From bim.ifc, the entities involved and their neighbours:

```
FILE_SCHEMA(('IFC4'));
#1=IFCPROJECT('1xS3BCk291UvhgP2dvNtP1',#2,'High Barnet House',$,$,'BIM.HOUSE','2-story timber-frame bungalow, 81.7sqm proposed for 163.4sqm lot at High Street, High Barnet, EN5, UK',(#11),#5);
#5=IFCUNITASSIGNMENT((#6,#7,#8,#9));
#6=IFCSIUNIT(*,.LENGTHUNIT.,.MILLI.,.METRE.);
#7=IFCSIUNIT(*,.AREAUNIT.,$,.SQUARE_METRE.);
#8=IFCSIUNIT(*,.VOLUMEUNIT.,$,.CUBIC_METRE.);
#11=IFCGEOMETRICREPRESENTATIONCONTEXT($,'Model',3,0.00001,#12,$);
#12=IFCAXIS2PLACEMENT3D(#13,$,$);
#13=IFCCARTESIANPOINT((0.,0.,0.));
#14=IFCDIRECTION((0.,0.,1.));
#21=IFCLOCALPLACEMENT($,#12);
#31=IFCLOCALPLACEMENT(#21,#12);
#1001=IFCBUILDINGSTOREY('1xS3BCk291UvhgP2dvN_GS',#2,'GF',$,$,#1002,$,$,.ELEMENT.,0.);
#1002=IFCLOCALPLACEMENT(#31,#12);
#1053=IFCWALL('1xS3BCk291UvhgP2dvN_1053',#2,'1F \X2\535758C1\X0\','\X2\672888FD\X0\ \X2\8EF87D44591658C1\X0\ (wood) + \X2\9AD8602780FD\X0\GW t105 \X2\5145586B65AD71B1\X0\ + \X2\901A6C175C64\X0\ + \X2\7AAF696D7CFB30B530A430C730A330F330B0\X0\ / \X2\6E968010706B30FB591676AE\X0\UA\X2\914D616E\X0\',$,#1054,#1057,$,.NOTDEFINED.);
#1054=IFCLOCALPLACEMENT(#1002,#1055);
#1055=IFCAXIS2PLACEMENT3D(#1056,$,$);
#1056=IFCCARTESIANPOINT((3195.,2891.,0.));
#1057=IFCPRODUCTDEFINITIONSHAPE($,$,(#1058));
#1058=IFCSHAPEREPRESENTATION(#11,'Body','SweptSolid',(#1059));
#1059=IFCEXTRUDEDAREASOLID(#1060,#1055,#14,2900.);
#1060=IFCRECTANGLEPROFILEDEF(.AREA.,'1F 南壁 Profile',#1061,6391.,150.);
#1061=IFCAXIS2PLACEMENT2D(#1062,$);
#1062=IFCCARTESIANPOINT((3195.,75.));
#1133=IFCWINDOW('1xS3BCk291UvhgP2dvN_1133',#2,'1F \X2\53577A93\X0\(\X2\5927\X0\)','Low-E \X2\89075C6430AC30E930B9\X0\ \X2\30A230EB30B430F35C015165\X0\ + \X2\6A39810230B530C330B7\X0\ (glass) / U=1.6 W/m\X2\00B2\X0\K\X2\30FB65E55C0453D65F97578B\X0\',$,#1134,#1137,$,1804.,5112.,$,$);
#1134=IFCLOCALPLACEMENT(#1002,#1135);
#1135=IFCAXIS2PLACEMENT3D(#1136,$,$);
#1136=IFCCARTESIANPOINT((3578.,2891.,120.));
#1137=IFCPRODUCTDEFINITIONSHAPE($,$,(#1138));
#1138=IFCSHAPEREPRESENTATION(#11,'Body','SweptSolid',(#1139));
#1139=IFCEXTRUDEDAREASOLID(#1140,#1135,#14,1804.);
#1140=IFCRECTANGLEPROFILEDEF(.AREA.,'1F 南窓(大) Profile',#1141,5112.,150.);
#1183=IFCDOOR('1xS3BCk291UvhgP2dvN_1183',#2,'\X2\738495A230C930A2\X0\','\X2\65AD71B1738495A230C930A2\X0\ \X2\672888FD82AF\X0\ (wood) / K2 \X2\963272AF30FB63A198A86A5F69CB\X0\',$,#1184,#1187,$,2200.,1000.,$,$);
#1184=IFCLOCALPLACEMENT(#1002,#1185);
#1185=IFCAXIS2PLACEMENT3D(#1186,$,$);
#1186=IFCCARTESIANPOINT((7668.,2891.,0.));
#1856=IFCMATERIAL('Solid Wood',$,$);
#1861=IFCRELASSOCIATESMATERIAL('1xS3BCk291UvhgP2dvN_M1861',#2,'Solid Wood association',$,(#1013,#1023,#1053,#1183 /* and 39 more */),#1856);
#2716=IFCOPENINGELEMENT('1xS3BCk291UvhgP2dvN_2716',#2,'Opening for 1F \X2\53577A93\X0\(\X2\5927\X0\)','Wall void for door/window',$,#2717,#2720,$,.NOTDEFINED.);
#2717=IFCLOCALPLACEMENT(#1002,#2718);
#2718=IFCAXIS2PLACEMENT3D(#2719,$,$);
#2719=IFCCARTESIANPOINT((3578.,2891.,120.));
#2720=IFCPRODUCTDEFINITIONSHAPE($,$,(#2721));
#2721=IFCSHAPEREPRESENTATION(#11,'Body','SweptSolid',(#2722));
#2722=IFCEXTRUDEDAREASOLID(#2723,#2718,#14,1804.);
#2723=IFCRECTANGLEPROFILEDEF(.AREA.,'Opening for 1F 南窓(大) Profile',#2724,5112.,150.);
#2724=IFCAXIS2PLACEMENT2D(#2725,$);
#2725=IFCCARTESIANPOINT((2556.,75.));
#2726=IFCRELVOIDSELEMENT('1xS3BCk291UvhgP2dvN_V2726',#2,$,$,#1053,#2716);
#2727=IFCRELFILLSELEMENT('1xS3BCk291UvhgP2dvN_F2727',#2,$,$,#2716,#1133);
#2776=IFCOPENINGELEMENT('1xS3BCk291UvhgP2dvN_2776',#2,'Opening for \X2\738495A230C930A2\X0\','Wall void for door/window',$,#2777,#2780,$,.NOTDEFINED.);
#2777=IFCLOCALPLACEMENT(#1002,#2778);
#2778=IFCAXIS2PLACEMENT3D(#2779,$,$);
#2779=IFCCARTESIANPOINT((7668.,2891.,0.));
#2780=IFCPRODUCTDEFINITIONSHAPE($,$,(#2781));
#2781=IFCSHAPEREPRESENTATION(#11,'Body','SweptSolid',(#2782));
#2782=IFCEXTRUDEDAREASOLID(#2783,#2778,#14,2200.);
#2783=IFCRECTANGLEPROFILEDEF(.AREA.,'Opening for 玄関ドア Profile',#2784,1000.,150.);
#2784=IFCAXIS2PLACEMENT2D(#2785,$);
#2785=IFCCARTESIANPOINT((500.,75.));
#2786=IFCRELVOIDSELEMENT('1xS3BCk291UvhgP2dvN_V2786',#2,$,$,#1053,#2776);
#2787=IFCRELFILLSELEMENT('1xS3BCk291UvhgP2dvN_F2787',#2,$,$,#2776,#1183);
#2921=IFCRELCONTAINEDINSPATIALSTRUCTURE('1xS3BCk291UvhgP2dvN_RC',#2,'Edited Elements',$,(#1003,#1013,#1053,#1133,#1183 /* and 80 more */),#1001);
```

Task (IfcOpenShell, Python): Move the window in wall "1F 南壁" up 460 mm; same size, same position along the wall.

```python
import numpy as np
import ifcopenshell
import ifcopenshell.api.geometry
import ifcopenshell.util.placement
import ifcopenshell.util.unit

model = ifcopenshell.open("bim.ifc")
unit_scale = ifcopenshell.util.unit.calculate_unit_scale(model)

window = model.by_guid("1xS3BCk291UvhgP2dvN_1133")
opening = window.FillsVoids[0].RelatingOpeningElement
dz = 0.46 / unit_scale

shift = np.array([0.0, 0.0, dz])
# The window is not placed relative to its opening, so move both.
for product in (opening, window):
    matrix = ifcopenshell.util.placement.get_local_placement(product.ObjectPlacement)
    matrix[:3, 3] += shift
    ifcopenshell.api.geometry.edit_object_placement(model, product=product, matrix=matrix, is_si=False)

print(f"moved by {dz * unit_scale:+.3f} m")

model.write("bim_updated.ifc")
```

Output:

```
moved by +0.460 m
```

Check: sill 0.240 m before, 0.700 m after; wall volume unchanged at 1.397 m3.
